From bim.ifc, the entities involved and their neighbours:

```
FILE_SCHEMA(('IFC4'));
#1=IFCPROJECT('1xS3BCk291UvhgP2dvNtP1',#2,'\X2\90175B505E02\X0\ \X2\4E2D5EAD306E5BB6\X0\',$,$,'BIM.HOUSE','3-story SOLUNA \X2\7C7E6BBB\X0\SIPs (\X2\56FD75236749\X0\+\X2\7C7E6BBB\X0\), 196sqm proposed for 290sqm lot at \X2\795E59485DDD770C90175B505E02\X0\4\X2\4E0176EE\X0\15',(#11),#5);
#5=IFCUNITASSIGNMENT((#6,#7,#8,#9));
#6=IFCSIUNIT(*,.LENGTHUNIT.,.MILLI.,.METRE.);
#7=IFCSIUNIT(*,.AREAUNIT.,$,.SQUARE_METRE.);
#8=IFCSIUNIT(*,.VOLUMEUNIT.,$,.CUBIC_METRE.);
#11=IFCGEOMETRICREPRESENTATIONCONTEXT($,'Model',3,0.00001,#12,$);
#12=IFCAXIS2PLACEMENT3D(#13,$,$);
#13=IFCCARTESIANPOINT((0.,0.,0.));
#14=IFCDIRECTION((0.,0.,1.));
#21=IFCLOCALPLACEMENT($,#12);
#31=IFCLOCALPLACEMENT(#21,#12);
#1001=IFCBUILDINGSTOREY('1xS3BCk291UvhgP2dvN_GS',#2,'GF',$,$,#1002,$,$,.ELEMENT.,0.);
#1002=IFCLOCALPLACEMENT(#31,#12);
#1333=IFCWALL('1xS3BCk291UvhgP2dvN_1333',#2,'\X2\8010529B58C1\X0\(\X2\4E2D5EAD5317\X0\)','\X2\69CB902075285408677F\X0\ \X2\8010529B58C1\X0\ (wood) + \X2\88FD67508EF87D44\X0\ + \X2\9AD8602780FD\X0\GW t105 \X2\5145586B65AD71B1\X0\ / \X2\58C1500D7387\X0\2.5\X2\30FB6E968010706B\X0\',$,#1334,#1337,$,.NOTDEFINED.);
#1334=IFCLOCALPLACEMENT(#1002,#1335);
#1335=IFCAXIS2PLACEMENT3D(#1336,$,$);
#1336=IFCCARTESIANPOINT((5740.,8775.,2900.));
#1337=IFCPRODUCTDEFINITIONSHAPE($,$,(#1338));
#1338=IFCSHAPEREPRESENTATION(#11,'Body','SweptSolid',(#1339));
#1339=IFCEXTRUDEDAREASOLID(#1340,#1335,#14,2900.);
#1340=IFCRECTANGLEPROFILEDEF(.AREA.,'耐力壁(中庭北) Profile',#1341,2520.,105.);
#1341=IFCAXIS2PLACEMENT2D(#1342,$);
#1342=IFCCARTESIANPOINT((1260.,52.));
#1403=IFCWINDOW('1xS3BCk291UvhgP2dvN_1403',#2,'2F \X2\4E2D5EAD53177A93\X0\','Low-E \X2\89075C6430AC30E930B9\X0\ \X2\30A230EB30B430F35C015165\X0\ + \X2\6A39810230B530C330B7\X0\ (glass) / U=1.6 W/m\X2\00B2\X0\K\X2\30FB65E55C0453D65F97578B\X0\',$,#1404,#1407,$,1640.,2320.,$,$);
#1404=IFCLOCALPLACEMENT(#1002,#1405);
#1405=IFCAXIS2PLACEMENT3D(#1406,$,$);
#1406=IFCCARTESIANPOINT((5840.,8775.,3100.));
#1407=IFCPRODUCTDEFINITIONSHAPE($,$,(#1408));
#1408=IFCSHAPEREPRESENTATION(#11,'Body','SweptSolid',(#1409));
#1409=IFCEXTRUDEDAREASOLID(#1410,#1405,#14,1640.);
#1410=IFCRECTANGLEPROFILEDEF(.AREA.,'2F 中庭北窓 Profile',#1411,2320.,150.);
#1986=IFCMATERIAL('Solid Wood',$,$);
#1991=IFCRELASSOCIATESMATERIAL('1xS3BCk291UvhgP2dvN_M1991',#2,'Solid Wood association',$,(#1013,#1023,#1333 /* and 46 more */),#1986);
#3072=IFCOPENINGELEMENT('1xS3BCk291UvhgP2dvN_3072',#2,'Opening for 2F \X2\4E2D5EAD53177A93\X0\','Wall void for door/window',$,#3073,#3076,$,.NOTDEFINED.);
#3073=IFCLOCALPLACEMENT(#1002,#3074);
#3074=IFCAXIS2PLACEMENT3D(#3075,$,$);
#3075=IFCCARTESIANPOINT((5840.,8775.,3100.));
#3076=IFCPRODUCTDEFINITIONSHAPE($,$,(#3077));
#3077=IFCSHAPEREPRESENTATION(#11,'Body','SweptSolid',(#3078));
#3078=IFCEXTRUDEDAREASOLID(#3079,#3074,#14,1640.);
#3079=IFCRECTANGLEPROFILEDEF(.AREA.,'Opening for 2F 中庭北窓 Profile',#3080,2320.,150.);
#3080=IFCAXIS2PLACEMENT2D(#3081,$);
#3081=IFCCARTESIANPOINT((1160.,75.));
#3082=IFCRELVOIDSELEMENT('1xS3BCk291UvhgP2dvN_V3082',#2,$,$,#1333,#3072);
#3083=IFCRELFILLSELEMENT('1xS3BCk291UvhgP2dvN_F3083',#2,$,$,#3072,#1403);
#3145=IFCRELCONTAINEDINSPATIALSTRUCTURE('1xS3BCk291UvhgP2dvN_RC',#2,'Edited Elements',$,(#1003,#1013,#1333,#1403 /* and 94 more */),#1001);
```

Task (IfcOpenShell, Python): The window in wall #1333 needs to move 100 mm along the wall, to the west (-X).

```python
import ifcopenshell
import ifcopenshell.api.geometry
import ifcopenshell.util.placement
import ifcopenshell.util.unit

model = ifcopenshell.open("bim.ifc")
unit_scale = ifcopenshell.util.unit.calculate_unit_scale(model)

window = model.by_guid("1xS3BCk291UvhgP2dvN_1403")
opening = window.FillsVoids[0].RelatingOpeningElement
wall = opening.VoidsElements[0].RelatingBuildingElement

wall_matrix = ifcopenshell.util.placement.get_local_placement(wall.ObjectPlacement)
shift = wall_matrix[:3, 0] * -0.1 / unit_scale
before = ifcopenshell.util.placement.get_local_placement(window.ObjectPlacement)[:3, 3].copy()

# The window is not placed relative to its opening, so move both.
for product in (opening, window):
    matrix = ifcopenshell.util.placement.get_local_placement(product.ObjectPlacement)
    matrix[:3, 3] += shift
    ifcopenshell.api.geometry.edit_object_placement(model, product=product, matrix=matrix, is_si=False)

after = ifcopenshell.util.placement.get_local_placement(window.ObjectPlacement)[:3, 3]
print("window moved by", (after - before).round(3) + 0.0)

model.write("bim_rev.ifc")
```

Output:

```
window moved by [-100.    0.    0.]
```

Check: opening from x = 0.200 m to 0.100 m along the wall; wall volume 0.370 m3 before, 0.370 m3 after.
